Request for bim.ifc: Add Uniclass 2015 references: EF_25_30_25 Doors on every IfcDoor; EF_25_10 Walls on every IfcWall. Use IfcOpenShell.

First a look at what the model holds.

```python
import ifcopenshell

model = ifcopenshell.open("bim.ifc")
print(model.schema)
print("classifications:", [c.Name for c in model.by_type("IfcClassification")])
for ifc_class in ("IfcDoor", "IfcRoof", "IfcStair", "IfcWall", "IfcWindow"):
    print(ifc_class, len(model.by_type(ifc_class)))
```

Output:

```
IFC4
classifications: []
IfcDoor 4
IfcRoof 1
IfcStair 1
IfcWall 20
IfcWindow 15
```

```python
import ifcopenshell
import ifcopenshell.api.classification

model = ifcopenshell.open("bim.ifc")

system = ifcopenshell.api.classification.add_classification(model, classification="Uniclass 2015")

codes = {
    "IfcDoor": ("EF_25_30_25", "Doors"),
    "IfcWall": ("EF_25_10", "Walls"),
}
for ifc_class, (code, name) in codes.items():
    products = model.by_type(ifc_class)
    ifcopenshell.api.classification.add_reference(
        model, products=products, classification=system, identification=code, name=name
    )
    print(code, len(products))

model.write("bim_v2.ifc")
```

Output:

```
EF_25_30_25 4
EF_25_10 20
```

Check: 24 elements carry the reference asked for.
